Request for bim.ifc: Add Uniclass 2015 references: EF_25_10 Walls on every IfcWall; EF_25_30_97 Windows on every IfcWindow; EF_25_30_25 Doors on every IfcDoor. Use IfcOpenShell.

First a look at what the model holds.

```python
import ifcopenshell

model = ifcopenshell.open("bim.ifc")
print(model.schema)
print("classifications:", [c.Name for c in model.by_type("IfcClassification")])
for ifc_class in ("IfcDoor", "IfcRoof", "IfcStair", "IfcWall", "IfcWindow"):
    print(ifc_class, len(model.by_type(ifc_class)))
```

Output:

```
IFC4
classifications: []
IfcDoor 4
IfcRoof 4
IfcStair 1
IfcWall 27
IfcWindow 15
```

```python
import ifcopenshell
import ifcopenshell.api.classification

model = ifcopenshell.open("bim.ifc")

system = ifcopenshell.api.classification.add_classification(model, classification="Uniclass 2015")

codes = {
    "IfcWall": ("EF_25_10", "Walls"),
    "IfcWindow": ("EF_25_30_97", "Windows"),
    "IfcDoor": ("EF_25_30_25", "Doors"),
}
for ifc_class, (code, name) in codes.items():
    products = model.by_type(ifc_class)
    ifcopenshell.api.classification.add_reference(
        model, products=products, classification=system, identification=code, name=name
    )
    print(code, len(products))

model.write("bim_edited.ifc")
```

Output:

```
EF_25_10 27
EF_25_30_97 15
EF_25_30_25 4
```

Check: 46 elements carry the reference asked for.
